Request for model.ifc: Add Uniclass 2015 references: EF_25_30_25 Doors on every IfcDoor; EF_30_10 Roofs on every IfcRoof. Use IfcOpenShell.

First a look at what the model holds.

```python
import ifcopenshell

model = ifcopenshell.open("model.ifc")
print(model.schema)
print("classifications:", [c.Name for c in model.by_type("IfcClassification")])
for ifc_class in ("IfcDoor", "IfcRoof", "IfcStair", "IfcWall", "IfcWindow"):
    print(ifc_class, len(model.by_type(ifc_class)))
```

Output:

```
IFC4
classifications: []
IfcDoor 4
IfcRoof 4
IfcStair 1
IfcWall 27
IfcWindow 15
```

```python
import ifcopenshell
import ifcopenshell.api.classification

model = ifcopenshell.open("model.ifc")

system = ifcopenshell.api.classification.add_classification(model, classification="Uniclass 2015")

codes = {
    "IfcDoor": ("EF_25_30_25", "Doors"),
    "IfcRoof": ("EF_30_10", "Roofs"),
}
for ifc_class, (code, name) in codes.items():
    products = model.by_type(ifc_class)
    ifcopenshell.api.classification.add_reference(
        model, products=products, classification=system, identification=code, name=name
    )
    print(code, len(products))

model.write("model_v2.ifc")
```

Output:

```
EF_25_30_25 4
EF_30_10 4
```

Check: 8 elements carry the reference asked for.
